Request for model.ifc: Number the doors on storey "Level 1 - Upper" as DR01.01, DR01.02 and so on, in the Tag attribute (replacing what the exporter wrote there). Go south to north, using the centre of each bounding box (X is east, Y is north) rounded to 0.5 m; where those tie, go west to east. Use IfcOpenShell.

First a look at what the model holds.

```python
import ifcopenshell
import ifcopenshell.util.element
import ifcopenshell.util.placement

model = ifcopenshell.open("model.ifc")
print(model.schema)
storey = next(s for s in model.by_type("IfcBuildingStorey") if s.Name == "Level 1 - Upper")
doors = [e for e in ifcopenshell.util.element.get_decomposition(storey) if e.is_a("IfcDoor")]
for e in sorted(doors, key=lambda e: e.id()):
    origin = ifcopenshell.util.placement.get_local_placement(e.ObjectPlacement)[:3, 3]
    print(e.id(), e.Tag, e.Name, origin.round(2) + 0.0, sep=" | ")
```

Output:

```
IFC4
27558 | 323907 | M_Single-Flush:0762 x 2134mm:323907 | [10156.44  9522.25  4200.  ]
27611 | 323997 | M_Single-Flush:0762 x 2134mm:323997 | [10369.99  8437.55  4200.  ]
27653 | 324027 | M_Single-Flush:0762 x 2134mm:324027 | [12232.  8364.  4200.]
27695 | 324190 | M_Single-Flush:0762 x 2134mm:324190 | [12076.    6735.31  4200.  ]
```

```python
import ifcopenshell
import ifcopenshell.geom
import ifcopenshell.util.element
import ifcopenshell.util.shape

model = ifcopenshell.open("model.ifc")
settings = ifcopenshell.geom.settings()
settings.set("use-world-coords", True)


def centre(element):
    shape = ifcopenshell.geom.create_shape(settings, element)
    return ifcopenshell.util.shape.get_bbox_centroid(shape.geometry)


storey = next(s for s in model.by_type("IfcBuildingStorey") if s.Name == "Level 1 - Upper")
doors = [e for e in ifcopenshell.util.element.get_decomposition(storey) if e.is_a("IfcDoor")]

# Insertion points can sit at a corner or the storey origin, so sort by the geometry (in metres).
centres = {e: centre(e) for e in doors}
doors.sort(key=lambda e: (round(centres[e][1] / 0.5), centres[e][0]))

for i, e in enumerate(doors, start=1):
    number = f"DR01.{i:02d}"
    e.Tag = number
    print(e.id(), number)

model.write("model-out.ifc")
```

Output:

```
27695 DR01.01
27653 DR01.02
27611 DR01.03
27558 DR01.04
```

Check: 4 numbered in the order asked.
